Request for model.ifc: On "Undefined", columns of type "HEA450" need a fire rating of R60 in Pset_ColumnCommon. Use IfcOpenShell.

First a look at what the model holds.

```python
import ifcopenshell
import ifcopenshell.util.element

model = ifcopenshell.open("model.ifc")
print(model.schema)
storey = next(s for s in model.by_type("IfcBuildingStorey") if s.Name == "Undefined")
columns = [e for e in ifcopenshell.util.element.get_decomposition(storey) if e.is_a("IfcColumn")]
seen = {}
for e in columns:
    element_type = ifcopenshell.util.element.get_type(e)
    key = (element_type.Name if element_type != e and element_type else None, ifcopenshell.util.element.get_pset(e, "Pset_ColumnCommon", "FireRating"))
    seen[key] = seen.get(key, 0) + 1
for (name, value), count in sorted(seen.items(), key=str):
    print(count, "x", name, "|", value)
```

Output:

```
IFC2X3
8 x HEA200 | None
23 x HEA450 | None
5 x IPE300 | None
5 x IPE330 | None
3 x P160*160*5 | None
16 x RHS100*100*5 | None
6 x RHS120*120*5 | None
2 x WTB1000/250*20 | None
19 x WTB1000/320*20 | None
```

```python
import ifcopenshell
import ifcopenshell.api.pset
import ifcopenshell.util.element

model = ifcopenshell.open("model.ifc")

storey = next(s for s in model.by_type("IfcBuildingStorey") if s.Name == "Undefined")
columns = [e for e in ifcopenshell.util.element.get_decomposition(storey) if e.is_a("IfcColumn")]

count = 0
for e in columns:
    element_type = ifcopenshell.util.element.get_type(e)
    if element_type in (None, e) or element_type.Name != "HEA450":
        continue
    found = ifcopenshell.util.element.get_pset(e, "Pset_ColumnCommon", should_inherit=False)
    if found:
        pset = model.by_id(found["id"])
        if len(ifcopenshell.util.element.get_elements_by_pset(pset)) > 1:
            pset = ifcopenshell.api.pset.unshare_pset(model, products=[e], pset=pset)[0]
    else:
        pset = ifcopenshell.api.pset.add_pset(model, product=e, name="Pset_ColumnCommon")
    ifcopenshell.api.pset.edit_pset(model, pset=pset, properties={"FireRating": "R60"})
    count += 1

print(count, "columns updated")

model.write("model_rev.ifc")
```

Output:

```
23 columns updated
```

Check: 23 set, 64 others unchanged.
